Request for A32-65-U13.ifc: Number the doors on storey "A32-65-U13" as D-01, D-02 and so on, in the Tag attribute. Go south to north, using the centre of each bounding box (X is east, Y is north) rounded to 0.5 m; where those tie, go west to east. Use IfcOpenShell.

First a look at what the model holds.

```python
import ifcopenshell
import ifcopenshell.util.element
import ifcopenshell.util.placement

model = ifcopenshell.open("A32-65-U13.ifc")
print(model.schema)
storey = next(s for s in model.by_type("IfcBuildingStorey") if s.Name == "A32-65-U13")
doors = [e for e in ifcopenshell.util.element.get_decomposition(storey) if e.is_a("IfcDoor")]
for e in sorted(doors, key=lambda e: e.id()):
    origin = ifcopenshell.util.placement.get_local_placement(e.ObjectPlacement)[:3, 3]
    print(e.id(), e.Tag, e.Name, origin.round(2) + 0.0, sep=" | ")
```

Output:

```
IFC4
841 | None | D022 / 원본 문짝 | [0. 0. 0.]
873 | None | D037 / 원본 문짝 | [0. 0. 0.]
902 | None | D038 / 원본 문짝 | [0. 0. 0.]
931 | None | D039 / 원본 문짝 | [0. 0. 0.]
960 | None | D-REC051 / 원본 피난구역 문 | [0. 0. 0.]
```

```python
import ifcopenshell
import ifcopenshell.geom
import ifcopenshell.util.element
import ifcopenshell.util.shape

model = ifcopenshell.open("A32-65-U13.ifc")
settings = ifcopenshell.geom.settings()
settings.set("use-world-coords", True)


def centre(element):
    shape = ifcopenshell.geom.create_shape(settings, element)
    return ifcopenshell.util.shape.get_bbox_centroid(shape.geometry)


storey = next(s for s in model.by_type("IfcBuildingStorey") if s.Name == "A32-65-U13")
doors = [e for e in ifcopenshell.util.element.get_decomposition(storey) if e.is_a("IfcDoor")]

# Insertion points can sit at a corner or the storey origin, so sort by the geometry (in metres).
centres = {e: centre(e) for e in doors}
doors.sort(key=lambda e: (round(centres[e][1] / 0.5), centres[e][0]))

for i, e in enumerate(doors, start=1):
    number = f"D-{i:02d}"
    e.Tag = number
    print(e.id(), number)

model.write("A32-65-U13_updated.ifc")
```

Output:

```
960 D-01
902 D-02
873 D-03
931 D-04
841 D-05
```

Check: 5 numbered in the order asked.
